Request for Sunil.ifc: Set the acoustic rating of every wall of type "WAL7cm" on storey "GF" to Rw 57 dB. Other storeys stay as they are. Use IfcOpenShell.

First a look at what the model holds.

```python
import ifcopenshell
import ifcopenshell.util.element

model = ifcopenshell.open("Sunil.ifc")
print(model.schema)
storey = next(s for s in model.by_type("IfcBuildingStorey") if s.Name == "GF")
walls = [e for e in ifcopenshell.util.element.get_decomposition(storey) if e.is_a("IfcWall")]
seen = {}
for e in walls:
    element_type = ifcopenshell.util.element.get_type(e)
    key = (element_type.Name if element_type != e and element_type else None, ifcopenshell.util.element.get_pset(e, "Pset_WallCommon", "AcousticRating"))
    seen[key] = seen.get(key, 0) + 1
for (name, value), count in sorted(seen.items(), key=str):
    print(count, "x", name, "|", value)
```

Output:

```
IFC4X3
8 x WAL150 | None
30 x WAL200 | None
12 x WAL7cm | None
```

```python
import ifcopenshell
import ifcopenshell.api.pset
import ifcopenshell.util.element

model = ifcopenshell.open("Sunil.ifc")

storey = next(s for s in model.by_type("IfcBuildingStorey") if s.Name == "GF")
walls = [e for e in ifcopenshell.util.element.get_decomposition(storey) if e.is_a("IfcWall")]

count = 0
for e in walls:
    element_type = ifcopenshell.util.element.get_type(e)
    if element_type in (None, e) or element_type.Name != "WAL7cm":
        continue
    # add_pset returns the element's existing set when there is one.
    pset = ifcopenshell.api.pset.add_pset(model, product=e, name="Pset_WallCommon")
    ifcopenshell.api.pset.edit_pset(model, pset=pset, properties={"AcousticRating": "Rw 57 dB"})
    count += 1

print(count, "walls updated")

model.write("Sunil_v2.ifc")
```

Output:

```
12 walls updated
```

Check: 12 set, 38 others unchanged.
